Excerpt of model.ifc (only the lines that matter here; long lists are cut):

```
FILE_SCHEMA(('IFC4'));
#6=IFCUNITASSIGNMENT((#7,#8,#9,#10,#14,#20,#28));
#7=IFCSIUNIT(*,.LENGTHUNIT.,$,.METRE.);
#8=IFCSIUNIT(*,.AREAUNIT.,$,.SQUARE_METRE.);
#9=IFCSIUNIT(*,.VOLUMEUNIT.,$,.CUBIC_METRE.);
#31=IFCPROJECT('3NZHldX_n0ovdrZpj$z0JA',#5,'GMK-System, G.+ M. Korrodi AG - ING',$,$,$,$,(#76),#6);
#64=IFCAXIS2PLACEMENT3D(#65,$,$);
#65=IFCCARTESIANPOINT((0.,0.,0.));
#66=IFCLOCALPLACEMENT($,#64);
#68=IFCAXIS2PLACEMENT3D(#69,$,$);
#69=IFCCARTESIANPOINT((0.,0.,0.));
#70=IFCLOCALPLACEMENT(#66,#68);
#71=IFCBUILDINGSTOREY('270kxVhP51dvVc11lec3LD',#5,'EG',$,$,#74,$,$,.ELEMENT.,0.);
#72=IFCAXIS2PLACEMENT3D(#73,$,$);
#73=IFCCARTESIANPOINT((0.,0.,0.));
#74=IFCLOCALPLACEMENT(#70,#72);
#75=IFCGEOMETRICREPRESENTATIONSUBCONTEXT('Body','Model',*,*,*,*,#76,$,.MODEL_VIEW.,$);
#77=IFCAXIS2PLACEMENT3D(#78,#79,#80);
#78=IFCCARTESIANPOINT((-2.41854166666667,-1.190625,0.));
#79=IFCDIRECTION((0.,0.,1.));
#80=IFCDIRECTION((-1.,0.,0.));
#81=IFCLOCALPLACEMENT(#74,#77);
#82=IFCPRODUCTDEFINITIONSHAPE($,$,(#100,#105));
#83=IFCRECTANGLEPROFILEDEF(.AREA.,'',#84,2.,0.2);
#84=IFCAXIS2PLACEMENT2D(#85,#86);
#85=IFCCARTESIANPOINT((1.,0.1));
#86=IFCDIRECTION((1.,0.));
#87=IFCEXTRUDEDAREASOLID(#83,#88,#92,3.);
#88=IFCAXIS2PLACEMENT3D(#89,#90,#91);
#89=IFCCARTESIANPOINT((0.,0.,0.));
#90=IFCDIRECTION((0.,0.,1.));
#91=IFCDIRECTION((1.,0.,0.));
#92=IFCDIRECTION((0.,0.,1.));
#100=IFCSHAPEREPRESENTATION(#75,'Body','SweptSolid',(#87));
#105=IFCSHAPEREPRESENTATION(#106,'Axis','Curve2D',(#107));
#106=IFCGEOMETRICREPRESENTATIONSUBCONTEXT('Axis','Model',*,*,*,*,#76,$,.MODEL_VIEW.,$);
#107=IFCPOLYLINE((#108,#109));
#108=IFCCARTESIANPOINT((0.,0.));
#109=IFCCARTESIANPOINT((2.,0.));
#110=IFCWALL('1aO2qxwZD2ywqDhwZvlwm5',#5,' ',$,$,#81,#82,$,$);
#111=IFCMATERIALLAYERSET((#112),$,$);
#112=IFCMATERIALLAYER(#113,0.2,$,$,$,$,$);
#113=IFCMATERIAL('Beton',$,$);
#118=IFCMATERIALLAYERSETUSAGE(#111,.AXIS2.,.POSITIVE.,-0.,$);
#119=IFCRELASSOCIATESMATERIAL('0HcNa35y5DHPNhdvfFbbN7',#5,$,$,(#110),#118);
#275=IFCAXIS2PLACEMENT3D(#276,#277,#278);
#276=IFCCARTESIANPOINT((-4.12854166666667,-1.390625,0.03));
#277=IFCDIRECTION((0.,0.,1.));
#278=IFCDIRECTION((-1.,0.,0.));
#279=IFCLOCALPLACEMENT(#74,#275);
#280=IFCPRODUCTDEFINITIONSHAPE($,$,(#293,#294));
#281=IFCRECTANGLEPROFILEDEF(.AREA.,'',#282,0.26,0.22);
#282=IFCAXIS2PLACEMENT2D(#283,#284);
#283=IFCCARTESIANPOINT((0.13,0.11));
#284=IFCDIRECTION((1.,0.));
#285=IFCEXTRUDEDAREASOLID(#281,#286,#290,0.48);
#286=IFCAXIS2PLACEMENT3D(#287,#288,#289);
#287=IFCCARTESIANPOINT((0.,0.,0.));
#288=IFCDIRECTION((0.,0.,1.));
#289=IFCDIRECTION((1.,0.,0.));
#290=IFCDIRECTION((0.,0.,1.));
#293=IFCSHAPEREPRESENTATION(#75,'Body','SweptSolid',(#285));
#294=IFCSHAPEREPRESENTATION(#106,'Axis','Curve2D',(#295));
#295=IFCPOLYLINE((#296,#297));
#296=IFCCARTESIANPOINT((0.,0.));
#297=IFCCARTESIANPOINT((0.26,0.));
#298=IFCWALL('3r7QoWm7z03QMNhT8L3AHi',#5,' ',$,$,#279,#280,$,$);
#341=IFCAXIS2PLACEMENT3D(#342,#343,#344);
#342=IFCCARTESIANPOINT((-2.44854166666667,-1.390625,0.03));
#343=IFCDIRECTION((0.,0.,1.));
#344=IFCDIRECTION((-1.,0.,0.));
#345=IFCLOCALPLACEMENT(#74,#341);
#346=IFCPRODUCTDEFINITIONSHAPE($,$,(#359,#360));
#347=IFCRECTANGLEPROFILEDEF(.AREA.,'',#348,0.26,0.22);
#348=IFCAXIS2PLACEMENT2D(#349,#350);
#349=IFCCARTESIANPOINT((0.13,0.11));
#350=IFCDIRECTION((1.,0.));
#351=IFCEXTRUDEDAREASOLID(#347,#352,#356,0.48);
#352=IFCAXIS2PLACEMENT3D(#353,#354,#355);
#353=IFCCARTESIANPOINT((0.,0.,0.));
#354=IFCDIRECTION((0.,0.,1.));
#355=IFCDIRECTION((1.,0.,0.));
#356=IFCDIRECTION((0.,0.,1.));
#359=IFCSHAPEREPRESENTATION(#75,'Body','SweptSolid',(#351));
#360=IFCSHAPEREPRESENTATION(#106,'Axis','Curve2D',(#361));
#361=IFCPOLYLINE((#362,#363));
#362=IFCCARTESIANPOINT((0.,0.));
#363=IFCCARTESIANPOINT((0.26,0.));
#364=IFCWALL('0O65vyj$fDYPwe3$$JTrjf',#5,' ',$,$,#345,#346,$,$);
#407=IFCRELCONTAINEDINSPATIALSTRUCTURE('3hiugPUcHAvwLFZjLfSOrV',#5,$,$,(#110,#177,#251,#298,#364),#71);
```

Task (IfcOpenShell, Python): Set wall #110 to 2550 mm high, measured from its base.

```python
import ifcopenshell
import ifcopenshell.geom
import ifcopenshell.util.representation
import ifcopenshell.util.shape

model = ifcopenshell.open("model.ifc")
settings = ifcopenshell.geom.settings()


def volume(element):
    """Net volume in cubic metres, openings subtracted."""
    shape = ifcopenshell.geom.create_shape(settings, element)
    return ifcopenshell.util.shape.get_volume(shape.geometry)


wall = model.by_guid("1aO2qxwZD2ywqDhwZvlwm5")
before = volume(wall)

body = ifcopenshell.util.representation.get_representation(wall, "Model", "Body")
solid = body.Items[0]
old_height = solid.Depth
solid.Depth = 2.55
after = volume(wall)

print(f"height {old_height:g} -> {solid.Depth:g}, volume {before:.3f} -> {after:.3f} m3")

model.write("model_rev.ifc")
```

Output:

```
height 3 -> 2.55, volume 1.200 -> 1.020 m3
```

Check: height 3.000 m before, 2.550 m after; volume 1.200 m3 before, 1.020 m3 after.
